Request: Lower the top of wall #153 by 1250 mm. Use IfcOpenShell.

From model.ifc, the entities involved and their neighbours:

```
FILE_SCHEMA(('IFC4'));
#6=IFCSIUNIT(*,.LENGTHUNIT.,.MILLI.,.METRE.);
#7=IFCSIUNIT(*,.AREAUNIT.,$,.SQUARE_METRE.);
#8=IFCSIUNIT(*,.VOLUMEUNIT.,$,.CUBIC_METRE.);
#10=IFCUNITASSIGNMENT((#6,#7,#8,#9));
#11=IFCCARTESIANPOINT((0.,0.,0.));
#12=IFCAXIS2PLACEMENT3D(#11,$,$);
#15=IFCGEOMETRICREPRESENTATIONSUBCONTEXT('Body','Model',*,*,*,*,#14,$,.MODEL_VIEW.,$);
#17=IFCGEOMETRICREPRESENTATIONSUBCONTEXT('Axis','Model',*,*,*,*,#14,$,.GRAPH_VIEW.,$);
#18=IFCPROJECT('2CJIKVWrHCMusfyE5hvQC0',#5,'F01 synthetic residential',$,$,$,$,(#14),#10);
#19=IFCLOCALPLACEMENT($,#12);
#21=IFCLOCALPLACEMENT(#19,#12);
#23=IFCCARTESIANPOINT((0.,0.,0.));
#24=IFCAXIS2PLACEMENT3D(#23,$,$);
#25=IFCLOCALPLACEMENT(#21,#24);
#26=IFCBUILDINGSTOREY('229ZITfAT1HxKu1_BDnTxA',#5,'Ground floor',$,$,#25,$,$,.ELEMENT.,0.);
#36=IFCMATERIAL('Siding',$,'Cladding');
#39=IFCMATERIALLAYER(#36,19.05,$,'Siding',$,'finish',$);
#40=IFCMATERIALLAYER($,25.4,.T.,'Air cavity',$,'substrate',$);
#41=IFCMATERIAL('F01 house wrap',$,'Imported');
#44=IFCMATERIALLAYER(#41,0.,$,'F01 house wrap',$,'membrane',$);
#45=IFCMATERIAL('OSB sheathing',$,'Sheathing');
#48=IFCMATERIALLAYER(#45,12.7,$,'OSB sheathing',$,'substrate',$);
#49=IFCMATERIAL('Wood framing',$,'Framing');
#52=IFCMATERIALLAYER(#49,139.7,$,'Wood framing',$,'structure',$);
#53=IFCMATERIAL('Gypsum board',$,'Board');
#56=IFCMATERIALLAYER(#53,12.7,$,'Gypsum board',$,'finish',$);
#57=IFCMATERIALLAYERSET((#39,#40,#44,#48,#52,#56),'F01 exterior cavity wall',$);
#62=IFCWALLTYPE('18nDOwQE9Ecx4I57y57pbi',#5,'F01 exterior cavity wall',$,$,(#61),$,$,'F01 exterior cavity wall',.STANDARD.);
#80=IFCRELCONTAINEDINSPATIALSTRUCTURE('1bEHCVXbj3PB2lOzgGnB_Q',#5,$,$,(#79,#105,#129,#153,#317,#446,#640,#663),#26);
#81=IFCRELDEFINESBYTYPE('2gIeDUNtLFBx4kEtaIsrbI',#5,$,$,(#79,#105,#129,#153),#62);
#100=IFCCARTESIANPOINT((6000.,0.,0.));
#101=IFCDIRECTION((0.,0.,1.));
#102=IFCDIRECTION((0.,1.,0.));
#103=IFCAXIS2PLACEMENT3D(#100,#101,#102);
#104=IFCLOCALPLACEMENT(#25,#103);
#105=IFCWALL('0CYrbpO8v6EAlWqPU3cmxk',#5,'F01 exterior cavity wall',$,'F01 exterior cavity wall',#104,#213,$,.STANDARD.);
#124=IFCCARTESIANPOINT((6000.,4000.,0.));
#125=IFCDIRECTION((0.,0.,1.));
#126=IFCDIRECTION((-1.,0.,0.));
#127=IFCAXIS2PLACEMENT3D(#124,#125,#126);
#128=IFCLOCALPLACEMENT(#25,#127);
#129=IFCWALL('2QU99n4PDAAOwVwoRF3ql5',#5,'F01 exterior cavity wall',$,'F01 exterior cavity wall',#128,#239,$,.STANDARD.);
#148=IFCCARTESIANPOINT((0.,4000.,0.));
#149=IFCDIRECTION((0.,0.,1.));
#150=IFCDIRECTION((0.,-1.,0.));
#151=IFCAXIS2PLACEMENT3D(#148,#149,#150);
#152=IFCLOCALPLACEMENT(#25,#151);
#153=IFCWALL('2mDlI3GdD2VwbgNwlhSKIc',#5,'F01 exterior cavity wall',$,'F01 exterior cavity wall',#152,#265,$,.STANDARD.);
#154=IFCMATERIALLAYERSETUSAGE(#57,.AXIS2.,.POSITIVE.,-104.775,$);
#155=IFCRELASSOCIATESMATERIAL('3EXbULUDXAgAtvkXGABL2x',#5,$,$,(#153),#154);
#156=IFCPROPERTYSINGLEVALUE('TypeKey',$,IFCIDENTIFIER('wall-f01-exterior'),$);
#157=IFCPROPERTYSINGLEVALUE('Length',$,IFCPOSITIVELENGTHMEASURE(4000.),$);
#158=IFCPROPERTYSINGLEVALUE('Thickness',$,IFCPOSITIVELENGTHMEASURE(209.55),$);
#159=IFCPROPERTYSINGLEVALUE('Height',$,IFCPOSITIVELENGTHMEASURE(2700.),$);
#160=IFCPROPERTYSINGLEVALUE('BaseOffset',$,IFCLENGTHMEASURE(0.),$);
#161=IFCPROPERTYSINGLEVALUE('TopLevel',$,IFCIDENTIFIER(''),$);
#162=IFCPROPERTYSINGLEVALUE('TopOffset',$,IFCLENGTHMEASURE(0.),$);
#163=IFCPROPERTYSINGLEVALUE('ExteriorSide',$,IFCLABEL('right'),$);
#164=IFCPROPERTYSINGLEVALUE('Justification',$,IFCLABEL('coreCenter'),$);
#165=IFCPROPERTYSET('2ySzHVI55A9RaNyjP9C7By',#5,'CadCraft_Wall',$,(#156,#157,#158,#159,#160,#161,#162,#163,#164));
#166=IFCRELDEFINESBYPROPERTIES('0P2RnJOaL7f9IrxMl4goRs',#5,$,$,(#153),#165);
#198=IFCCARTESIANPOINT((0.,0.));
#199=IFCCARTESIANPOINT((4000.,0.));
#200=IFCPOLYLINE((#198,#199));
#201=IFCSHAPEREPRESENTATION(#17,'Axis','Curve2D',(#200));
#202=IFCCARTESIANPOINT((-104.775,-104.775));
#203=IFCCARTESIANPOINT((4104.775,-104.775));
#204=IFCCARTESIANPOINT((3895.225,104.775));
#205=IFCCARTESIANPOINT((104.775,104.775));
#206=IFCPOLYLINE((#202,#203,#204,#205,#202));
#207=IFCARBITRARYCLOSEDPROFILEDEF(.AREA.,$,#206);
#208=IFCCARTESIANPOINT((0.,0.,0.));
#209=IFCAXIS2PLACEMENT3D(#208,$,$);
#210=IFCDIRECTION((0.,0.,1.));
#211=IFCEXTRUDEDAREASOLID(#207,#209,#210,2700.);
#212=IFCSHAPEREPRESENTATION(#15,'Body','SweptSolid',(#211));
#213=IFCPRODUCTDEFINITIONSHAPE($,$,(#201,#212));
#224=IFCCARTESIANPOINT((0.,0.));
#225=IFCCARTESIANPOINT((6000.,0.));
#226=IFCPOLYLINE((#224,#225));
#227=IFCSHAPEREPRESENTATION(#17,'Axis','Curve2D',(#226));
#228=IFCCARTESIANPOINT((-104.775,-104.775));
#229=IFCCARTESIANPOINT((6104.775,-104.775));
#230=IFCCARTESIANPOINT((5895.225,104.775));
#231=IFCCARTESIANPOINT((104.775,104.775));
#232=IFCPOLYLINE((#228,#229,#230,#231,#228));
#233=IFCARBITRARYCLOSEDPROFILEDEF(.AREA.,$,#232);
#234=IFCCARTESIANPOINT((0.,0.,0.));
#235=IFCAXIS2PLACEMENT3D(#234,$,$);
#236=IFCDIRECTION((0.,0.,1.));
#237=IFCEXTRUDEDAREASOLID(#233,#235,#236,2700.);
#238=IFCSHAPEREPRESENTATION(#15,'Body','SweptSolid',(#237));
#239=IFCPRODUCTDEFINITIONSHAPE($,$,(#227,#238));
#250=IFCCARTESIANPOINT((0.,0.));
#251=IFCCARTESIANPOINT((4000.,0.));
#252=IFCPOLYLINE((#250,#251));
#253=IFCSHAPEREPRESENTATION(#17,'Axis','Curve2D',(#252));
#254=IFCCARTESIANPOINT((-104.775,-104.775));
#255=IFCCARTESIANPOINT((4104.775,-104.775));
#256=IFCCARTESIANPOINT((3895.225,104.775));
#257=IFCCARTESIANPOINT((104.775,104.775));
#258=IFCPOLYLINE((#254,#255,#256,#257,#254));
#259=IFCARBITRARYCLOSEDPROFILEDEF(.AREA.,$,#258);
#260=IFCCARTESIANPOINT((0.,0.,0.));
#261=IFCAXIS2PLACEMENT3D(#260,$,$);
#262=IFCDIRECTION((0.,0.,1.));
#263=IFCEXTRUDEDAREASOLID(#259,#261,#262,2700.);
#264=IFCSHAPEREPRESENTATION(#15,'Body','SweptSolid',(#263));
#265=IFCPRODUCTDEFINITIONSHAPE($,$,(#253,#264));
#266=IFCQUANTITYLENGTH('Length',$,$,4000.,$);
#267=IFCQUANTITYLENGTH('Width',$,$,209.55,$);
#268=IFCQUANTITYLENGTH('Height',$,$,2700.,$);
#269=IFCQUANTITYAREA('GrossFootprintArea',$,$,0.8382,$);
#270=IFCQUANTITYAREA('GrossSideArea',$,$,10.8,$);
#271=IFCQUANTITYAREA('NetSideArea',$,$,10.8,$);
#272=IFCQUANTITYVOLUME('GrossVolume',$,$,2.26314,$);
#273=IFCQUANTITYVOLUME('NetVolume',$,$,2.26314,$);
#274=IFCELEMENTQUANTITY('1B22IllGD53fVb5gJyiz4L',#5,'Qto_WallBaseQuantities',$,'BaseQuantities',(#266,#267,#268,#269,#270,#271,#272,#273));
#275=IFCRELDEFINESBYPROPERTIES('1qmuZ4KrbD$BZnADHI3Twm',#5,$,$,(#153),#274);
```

```python
import ifcopenshell
import ifcopenshell.api.pset
import ifcopenshell.geom
import ifcopenshell.util.element
import ifcopenshell.util.representation
import ifcopenshell.util.shape
import ifcopenshell.util.unit

model = ifcopenshell.open("model.ifc")
unit_scale = ifcopenshell.util.unit.calculate_unit_scale(model)
area_scale = ifcopenshell.util.unit.calculate_unit_scale(model, "AREAUNIT")
volume_scale = ifcopenshell.util.unit.calculate_unit_scale(model, "VOLUMEUNIT")
settings = ifcopenshell.geom.settings()


def volume(element):
    """Net volume in cubic metres, openings subtracted."""
    shape = ifcopenshell.geom.create_shape(settings, element)
    return ifcopenshell.util.shape.get_volume(shape.geometry)


wall = model.by_id(153)
before = volume(wall)

body = ifcopenshell.util.representation.get_representation(wall, "Model", "Body")
solid = body.Items[0]
old_height = solid.Depth
solid.Depth -= 1.25 / unit_scale
after = volume(wall)
thickness = 0.2096  # wall thickness in metres

# Update the stored height, areas and volumes.
pset = model.by_id(ifcopenshell.util.element.get_pset(wall, "CadCraft_Wall", should_inherit=False)["id"])
ifcopenshell.api.pset.edit_pset(model, pset=pset, properties={
    "Height": model.create_entity("IfcPositiveLengthMeasure", solid.Depth),
})
qto = model.by_id(ifcopenshell.util.element.get_pset(wall, "Qto_WallBaseQuantities", should_inherit=False)["id"])
ifcopenshell.api.pset.edit_qto(model, qto=qto, properties={
    "Height": solid.Depth,
    "GrossSideArea": ifcopenshell.util.element.get_pset(wall, "Qto_WallBaseQuantities", "GrossSideArea") * solid.Depth / old_height,
    "NetSideArea": after / thickness / area_scale,
    "GrossVolume": ifcopenshell.util.element.get_pset(wall, "Qto_WallBaseQuantities", "GrossVolume") * solid.Depth / old_height,
    "NetVolume": after / volume_scale,
})

print(f"height {old_height:g} -> {solid.Depth:g}, volume {before:.3f} -> {after:.3f} m3")

model.write("model_edited.ifc")
```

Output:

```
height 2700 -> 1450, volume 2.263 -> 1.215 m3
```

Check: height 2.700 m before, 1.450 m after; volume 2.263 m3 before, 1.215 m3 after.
